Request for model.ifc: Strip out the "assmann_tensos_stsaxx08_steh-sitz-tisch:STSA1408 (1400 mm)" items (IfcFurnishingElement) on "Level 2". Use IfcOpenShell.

First a look at what the model holds.

```python
import ifcopenshell
import ifcopenshell.util.element

model = ifcopenshell.open("model.ifc")
print(model.schema)
storey = next(s for s in model.by_type("IfcBuildingStorey") if s.Name == "Level 2")
furniture = [e for e in ifcopenshell.util.element.get_decomposition(storey) if e.is_a("IfcFurnishingElement")]
seen = {}
for e in furniture:
    element_type = ifcopenshell.util.element.get_type(e)
    name = element_type.Name if element_type not in (None, e) else None
    seen[name] = seen.get(name, 0) + 1
for name, count in sorted(seen.items(), key=str):
    print(count, "x", name)
```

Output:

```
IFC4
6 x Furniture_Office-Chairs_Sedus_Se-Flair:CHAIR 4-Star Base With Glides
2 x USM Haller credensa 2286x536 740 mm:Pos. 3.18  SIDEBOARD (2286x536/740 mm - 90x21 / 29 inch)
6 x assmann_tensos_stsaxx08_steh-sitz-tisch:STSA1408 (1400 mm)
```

```python
import ifcopenshell
import ifcopenshell.api.root
import ifcopenshell.util.element

model = ifcopenshell.open("model.ifc")

storey = next(s for s in model.by_type("IfcBuildingStorey") if s.Name == "Level 2")
furniture = [e for e in ifcopenshell.util.element.get_decomposition(storey) if e.is_a("IfcFurnishingElement")]
targets = [e for e in furniture if (t := ifcopenshell.util.element.get_type(e)) not in (None, e) and t.Name == "assmann_tensos_stsaxx08_steh-sitz-tisch:STSA1408 (1400 mm)"]

for e in targets:
    ifcopenshell.api.root.remove_product(model, product=e)
print(len(targets), "removed")

model.write("model-out.ifc")
```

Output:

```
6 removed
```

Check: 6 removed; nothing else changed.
